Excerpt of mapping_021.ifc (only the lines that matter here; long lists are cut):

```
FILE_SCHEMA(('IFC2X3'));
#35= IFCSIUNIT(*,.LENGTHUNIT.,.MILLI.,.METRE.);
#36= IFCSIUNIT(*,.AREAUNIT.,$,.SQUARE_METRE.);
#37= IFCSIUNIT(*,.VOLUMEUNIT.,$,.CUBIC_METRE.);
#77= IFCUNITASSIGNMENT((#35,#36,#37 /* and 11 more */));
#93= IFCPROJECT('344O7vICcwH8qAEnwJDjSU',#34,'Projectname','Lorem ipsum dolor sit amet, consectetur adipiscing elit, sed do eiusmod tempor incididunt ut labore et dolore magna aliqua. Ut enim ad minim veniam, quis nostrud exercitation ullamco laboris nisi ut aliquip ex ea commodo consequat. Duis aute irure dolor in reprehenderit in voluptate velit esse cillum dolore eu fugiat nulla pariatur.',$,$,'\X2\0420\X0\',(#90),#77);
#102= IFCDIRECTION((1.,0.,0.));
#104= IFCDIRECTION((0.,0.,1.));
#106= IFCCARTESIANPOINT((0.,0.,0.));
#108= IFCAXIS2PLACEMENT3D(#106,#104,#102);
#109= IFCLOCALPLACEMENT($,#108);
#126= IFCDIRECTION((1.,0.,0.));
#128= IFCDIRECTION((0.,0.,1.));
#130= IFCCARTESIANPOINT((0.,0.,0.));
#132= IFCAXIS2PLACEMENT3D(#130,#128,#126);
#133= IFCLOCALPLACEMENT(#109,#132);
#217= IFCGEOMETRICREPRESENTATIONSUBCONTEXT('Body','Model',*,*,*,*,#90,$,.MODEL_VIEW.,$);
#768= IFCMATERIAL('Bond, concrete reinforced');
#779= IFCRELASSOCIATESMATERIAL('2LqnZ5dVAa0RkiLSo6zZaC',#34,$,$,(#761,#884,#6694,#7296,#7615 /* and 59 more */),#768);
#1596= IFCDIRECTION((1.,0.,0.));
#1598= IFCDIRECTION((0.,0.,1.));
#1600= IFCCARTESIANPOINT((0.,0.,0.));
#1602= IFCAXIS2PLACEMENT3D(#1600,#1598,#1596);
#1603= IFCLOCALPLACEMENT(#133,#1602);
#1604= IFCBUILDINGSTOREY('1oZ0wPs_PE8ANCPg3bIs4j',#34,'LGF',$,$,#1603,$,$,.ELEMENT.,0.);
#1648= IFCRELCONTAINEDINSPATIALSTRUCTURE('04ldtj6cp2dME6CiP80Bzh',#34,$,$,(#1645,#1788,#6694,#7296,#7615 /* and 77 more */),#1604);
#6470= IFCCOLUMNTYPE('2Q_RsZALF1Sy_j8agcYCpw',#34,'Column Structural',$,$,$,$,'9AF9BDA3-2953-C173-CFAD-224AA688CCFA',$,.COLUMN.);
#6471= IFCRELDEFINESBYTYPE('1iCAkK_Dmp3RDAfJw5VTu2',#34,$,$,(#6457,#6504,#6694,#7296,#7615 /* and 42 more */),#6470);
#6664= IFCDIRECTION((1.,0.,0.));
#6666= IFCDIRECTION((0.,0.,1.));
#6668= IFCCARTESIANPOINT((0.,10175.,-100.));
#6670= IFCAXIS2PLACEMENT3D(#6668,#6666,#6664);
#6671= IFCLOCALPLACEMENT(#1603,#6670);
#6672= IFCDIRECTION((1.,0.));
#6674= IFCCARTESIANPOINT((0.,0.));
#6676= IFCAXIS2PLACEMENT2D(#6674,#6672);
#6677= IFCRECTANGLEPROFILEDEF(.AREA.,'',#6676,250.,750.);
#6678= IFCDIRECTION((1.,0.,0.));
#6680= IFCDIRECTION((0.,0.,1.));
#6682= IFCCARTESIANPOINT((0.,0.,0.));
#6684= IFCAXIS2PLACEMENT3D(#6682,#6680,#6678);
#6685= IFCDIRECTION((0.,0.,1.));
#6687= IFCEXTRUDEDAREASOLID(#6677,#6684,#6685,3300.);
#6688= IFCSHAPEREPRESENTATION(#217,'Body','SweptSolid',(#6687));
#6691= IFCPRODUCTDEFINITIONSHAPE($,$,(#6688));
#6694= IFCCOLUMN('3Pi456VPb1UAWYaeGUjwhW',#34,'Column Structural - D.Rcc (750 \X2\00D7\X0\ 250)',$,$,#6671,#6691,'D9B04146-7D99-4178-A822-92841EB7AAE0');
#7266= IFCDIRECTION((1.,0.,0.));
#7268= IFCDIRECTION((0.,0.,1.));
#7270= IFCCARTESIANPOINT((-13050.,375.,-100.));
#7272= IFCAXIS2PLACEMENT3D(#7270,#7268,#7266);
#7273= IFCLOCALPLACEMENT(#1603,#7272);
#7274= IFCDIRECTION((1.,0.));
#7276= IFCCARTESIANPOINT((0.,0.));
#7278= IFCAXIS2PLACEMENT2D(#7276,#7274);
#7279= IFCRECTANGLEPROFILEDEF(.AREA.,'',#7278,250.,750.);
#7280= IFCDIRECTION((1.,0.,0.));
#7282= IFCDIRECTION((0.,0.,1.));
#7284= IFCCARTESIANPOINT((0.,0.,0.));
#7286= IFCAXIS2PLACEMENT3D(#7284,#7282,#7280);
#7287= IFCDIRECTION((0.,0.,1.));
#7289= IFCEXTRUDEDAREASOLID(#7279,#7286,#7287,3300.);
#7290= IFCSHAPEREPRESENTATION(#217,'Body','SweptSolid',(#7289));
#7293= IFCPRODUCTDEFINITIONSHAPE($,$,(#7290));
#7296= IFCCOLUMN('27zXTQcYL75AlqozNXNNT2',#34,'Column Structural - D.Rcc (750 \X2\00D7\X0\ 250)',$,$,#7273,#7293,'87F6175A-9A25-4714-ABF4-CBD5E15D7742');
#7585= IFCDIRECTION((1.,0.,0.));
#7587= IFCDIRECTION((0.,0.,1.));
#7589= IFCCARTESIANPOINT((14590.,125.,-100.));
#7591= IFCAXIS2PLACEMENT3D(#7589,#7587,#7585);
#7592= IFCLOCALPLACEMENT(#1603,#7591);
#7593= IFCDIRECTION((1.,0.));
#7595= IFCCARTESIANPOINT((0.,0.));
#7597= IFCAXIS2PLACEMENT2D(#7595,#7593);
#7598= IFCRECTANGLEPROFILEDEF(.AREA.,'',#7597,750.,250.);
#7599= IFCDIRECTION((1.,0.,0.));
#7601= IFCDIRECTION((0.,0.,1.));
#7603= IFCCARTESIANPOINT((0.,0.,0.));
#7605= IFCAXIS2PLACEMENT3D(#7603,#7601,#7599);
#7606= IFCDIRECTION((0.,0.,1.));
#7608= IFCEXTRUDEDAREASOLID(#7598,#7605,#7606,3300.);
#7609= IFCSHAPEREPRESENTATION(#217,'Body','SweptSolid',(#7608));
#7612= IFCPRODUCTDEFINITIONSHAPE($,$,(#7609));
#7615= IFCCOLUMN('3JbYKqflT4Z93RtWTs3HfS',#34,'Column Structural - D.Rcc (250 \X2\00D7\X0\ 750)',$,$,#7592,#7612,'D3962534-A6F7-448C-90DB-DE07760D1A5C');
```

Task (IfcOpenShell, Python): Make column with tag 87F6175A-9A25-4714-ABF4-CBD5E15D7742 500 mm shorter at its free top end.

```python
import ifcopenshell
import ifcopenshell.util.representation

model = ifcopenshell.open("mapping_021.ifc")

member = model.by_guid("27zXTQcYL75AlqozNXNNT2")
change = -500.0

# The extrusion runs towards the end named, so only its depth changes.
body = ifcopenshell.util.representation.get_representation(member, "Model", "Body")
solid = body.Items[0]
old_length = solid.Depth
solid.Depth += change

print(f"length {old_length:g} -> {solid.Depth:g}")

model.write("mapping_021-out.ifc")
```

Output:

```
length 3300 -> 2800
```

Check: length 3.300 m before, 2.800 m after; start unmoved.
